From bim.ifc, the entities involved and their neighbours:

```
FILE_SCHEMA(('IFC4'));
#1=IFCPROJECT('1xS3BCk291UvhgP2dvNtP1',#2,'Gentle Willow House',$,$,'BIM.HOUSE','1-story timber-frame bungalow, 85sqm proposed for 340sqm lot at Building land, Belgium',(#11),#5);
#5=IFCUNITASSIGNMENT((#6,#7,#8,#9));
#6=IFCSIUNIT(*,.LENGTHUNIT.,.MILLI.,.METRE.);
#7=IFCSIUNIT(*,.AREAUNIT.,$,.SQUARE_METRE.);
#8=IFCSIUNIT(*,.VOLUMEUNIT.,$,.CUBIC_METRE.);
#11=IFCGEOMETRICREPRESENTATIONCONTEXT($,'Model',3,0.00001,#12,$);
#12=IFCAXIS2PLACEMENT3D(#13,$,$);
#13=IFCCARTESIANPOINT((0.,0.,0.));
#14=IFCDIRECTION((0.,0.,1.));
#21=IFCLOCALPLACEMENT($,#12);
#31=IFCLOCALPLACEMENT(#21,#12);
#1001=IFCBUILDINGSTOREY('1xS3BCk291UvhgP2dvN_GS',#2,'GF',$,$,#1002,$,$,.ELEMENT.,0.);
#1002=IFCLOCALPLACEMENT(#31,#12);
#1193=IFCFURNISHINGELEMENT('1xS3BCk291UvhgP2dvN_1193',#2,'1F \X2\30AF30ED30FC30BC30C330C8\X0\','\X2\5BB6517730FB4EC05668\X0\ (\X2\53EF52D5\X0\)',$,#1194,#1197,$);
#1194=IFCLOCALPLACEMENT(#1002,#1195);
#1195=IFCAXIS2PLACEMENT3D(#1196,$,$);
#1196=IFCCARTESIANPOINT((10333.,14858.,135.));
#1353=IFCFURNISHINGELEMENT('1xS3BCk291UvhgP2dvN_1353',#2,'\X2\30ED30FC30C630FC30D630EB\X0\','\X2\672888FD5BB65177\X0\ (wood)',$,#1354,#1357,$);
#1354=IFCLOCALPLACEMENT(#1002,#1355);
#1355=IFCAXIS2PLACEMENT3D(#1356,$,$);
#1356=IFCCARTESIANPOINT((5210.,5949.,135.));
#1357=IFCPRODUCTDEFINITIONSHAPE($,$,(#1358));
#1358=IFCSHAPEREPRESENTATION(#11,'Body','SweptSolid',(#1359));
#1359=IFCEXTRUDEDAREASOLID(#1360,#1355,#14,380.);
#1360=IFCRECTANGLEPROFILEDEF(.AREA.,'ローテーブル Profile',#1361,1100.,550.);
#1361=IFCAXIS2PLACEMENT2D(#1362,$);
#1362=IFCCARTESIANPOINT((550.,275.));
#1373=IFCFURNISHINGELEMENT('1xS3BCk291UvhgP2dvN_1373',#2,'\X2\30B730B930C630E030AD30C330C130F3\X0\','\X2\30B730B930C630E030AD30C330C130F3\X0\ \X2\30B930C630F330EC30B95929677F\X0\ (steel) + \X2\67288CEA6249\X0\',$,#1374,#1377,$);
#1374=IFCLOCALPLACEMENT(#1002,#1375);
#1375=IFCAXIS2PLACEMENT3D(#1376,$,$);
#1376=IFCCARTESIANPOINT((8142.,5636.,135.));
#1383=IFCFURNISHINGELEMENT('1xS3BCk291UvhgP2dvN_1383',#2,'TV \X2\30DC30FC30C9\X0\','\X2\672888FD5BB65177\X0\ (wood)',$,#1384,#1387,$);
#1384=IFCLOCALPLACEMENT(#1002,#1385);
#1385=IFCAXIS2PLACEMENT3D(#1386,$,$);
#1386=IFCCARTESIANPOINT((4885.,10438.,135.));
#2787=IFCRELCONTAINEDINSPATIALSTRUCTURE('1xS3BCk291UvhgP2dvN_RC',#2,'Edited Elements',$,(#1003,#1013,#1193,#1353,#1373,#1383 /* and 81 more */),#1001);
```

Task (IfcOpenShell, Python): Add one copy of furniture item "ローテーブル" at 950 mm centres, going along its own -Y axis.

```python
import ifcopenshell
import ifcopenshell.api.geometry
import ifcopenshell.api.root
import ifcopenshell.util.element
import ifcopenshell.util.placement

model = ifcopenshell.open("bim.ifc")


def reuse_history(source, copy):
    """copy_class also copies each property set's owner history, people and application; keep the originals."""
    for rel in copy.IsDefinedBy:
        if rel.is_a("IfcRelDefinesByProperties") and (history := rel.RelatingPropertyDefinition.OwnerHistory):
            rel.RelatingPropertyDefinition.OwnerHistory = source.OwnerHistory
            ifcopenshell.util.element.remove_deep2(model, history)


source = model.by_guid("1xS3BCk291UvhgP2dvN_1353")
base = ifcopenshell.util.placement.get_local_placement(source.ObjectPlacement)
step = -base[:3, 1] * 950.0

for i in range(1, 2):
    copy = ifcopenshell.api.root.copy_class(model, product=source)
    copy.Representation = ifcopenshell.util.element.copy_deep(
        model, source.Representation, exclude=["IfcGeometricRepresentationContext", "IfcRepresentationMap"]
    )
    reuse_history(source, copy)
    matrix = base.copy()
    matrix[:3, 3] += i * step
    print("added at", matrix[:3, 3].round(3) + 0.0)
    ifcopenshell.api.geometry.edit_object_placement(model, product=copy, matrix=matrix, is_si=False)

model.write("bim_v2.ifc")
```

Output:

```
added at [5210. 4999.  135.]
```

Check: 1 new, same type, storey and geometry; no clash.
